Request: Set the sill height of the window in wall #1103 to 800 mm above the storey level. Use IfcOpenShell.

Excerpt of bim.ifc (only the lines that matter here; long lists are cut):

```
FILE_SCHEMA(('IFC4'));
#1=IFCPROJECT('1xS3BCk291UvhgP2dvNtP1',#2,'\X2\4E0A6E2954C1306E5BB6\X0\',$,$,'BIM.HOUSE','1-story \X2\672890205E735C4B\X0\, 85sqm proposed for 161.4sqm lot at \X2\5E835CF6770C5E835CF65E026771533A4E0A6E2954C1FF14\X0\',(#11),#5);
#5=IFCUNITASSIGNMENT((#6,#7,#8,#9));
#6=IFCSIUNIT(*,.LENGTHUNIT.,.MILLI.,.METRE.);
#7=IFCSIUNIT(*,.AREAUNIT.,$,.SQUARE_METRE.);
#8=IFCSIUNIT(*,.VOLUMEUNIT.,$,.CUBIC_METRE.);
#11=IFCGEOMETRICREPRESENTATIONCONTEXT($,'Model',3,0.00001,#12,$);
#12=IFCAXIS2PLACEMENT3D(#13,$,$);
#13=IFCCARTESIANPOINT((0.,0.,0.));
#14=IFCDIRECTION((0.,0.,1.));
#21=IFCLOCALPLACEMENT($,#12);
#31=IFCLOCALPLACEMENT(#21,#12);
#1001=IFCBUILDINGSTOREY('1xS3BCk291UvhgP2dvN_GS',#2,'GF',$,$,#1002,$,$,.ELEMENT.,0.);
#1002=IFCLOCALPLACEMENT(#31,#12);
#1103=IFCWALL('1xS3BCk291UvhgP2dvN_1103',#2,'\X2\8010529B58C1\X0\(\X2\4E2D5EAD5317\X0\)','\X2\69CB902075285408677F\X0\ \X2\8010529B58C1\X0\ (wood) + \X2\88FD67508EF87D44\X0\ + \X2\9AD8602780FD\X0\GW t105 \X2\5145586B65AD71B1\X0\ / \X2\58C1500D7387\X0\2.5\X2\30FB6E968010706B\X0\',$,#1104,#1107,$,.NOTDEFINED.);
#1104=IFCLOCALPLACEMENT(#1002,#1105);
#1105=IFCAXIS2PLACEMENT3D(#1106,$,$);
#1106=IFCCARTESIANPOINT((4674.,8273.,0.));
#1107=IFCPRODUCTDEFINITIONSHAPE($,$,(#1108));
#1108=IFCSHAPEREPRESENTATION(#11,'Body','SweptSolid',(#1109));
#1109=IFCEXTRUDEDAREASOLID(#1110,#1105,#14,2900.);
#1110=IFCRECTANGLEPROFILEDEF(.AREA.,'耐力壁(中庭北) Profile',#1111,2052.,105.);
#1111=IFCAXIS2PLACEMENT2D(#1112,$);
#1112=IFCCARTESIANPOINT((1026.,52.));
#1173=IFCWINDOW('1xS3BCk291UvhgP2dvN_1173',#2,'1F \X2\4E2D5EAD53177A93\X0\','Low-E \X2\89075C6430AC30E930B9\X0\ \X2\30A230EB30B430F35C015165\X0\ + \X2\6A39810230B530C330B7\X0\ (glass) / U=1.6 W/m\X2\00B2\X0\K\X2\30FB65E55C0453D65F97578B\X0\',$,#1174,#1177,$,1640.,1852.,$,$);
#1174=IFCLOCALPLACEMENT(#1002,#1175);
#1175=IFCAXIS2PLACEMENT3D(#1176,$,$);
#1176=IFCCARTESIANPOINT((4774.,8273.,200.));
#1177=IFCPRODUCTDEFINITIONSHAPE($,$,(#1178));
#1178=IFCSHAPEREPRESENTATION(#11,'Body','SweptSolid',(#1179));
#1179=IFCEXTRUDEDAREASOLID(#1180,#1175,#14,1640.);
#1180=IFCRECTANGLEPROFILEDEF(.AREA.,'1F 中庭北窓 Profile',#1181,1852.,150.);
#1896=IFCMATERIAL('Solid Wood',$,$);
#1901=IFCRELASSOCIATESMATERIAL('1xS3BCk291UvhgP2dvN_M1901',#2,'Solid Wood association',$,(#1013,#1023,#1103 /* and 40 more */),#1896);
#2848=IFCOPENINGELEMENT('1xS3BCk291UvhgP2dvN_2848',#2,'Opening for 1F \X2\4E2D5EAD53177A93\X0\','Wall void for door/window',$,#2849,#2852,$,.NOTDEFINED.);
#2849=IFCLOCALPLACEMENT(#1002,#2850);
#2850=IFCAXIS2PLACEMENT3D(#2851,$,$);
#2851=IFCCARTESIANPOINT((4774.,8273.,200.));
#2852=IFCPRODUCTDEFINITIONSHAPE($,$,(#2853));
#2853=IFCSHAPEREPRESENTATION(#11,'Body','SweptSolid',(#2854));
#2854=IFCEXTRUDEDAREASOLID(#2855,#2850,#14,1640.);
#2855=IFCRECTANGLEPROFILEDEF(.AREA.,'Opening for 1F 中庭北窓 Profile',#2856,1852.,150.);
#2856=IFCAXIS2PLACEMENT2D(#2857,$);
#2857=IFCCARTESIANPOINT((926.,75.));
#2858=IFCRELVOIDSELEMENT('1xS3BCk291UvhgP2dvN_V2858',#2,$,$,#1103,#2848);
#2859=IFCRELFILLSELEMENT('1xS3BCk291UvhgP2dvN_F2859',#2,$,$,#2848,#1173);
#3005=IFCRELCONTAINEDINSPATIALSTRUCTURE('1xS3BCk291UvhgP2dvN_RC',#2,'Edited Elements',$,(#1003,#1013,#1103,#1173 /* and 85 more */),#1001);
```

```python
import numpy as np
import ifcopenshell
import ifcopenshell.api.geometry
import ifcopenshell.geom
import ifcopenshell.util.element
import ifcopenshell.util.placement
import ifcopenshell.util.shape
import ifcopenshell.util.unit

model = ifcopenshell.open("bim.ifc")
unit_scale = ifcopenshell.util.unit.calculate_unit_scale(model)

window = model.by_id(1173)
opening = window.FillsVoids[0].RelatingOpeningElement
storey = ifcopenshell.util.element.get_container(window, ifc_class="IfcBuildingStorey")
level = ifcopenshell.util.placement.get_local_placement(storey.ObjectPlacement)[2, 3]

# The opening's origin need not be at the sill, so measure its lowest point.
shape = ifcopenshell.geom.create_shape(ifcopenshell.geom.settings(), opening)
bottom = ifcopenshell.util.shape.get_shape_bottom_elevation(shape, shape.geometry) / unit_scale
dz = level + 800.0 - bottom

shift = np.array([0.0, 0.0, dz])
# The window is not placed relative to its opening, so move both.
for product in (opening, window):
    matrix = ifcopenshell.util.placement.get_local_placement(product.ObjectPlacement)
    matrix[:3, 3] += shift
    ifcopenshell.api.geometry.edit_object_placement(model, product=product, matrix=matrix, is_si=False)

print(f"moved by {dz * unit_scale:+.3f} m")

model.write("bim_rev.ifc")
```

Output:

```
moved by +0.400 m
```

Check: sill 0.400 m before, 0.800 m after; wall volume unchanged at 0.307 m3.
